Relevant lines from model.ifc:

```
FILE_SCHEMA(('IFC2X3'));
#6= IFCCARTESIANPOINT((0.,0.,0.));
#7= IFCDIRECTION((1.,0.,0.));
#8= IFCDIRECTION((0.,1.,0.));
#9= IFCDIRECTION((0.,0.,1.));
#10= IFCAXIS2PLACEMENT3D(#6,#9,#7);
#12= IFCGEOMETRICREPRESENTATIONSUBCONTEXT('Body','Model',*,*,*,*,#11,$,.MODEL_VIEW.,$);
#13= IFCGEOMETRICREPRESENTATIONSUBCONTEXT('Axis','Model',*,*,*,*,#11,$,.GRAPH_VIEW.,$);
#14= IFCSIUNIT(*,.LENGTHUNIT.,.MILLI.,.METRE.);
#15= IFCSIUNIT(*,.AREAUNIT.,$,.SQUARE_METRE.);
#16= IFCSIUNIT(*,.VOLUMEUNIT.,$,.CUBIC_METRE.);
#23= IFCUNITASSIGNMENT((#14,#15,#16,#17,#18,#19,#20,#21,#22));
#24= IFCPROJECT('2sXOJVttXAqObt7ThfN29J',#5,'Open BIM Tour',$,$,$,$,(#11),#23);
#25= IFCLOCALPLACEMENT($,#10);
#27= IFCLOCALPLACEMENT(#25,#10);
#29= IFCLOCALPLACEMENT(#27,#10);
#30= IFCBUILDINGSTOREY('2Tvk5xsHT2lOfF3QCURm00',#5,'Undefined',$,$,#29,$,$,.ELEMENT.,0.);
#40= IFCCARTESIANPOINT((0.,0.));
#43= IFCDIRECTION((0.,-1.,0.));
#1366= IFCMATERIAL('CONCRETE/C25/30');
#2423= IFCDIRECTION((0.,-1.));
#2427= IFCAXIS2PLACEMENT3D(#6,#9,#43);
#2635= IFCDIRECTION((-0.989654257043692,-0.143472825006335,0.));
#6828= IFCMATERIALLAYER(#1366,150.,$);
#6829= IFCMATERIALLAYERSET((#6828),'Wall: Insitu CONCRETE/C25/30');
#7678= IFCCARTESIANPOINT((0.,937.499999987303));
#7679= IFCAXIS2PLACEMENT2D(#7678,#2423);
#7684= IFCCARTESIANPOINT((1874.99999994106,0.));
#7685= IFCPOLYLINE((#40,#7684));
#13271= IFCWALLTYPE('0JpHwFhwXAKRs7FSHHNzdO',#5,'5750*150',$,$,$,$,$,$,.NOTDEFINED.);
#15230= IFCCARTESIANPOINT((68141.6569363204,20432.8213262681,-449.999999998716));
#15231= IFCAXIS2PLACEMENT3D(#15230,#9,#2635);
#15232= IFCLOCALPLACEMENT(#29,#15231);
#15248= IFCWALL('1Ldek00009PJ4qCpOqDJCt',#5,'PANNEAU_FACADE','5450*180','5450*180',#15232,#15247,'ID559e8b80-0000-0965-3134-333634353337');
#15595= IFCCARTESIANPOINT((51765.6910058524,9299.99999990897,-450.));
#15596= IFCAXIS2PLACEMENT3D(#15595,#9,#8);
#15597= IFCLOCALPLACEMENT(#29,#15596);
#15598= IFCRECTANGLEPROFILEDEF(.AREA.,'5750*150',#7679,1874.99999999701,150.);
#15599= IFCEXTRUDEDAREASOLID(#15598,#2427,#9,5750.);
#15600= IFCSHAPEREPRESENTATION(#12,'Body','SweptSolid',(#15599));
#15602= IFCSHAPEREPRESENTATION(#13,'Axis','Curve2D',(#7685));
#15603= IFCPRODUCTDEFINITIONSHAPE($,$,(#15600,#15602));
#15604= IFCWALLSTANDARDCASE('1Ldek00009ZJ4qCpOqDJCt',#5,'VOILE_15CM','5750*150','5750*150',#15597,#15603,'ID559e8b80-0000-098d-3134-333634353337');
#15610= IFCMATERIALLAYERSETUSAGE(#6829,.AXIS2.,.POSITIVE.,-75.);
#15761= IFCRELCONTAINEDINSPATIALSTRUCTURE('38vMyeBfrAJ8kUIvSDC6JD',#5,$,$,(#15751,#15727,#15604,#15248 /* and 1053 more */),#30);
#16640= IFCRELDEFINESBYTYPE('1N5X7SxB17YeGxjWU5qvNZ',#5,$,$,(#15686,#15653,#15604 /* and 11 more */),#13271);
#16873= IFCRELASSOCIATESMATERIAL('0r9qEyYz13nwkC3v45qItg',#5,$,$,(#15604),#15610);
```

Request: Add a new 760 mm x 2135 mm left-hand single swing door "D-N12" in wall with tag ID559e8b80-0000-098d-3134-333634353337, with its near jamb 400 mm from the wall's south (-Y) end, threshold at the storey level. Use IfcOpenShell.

```python
import numpy as np
import ifcopenshell
import ifcopenshell.api.feature
import ifcopenshell.api.geometry
import ifcopenshell.api.root
import ifcopenshell.api.spatial
import ifcopenshell.api.type
import ifcopenshell.geom
import ifcopenshell.util.element
import ifcopenshell.util.placement
import ifcopenshell.util.representation
import ifcopenshell.util.shape
import ifcopenshell.util.unit

model = ifcopenshell.open("model.ifc")
unit_scale = ifcopenshell.util.unit.calculate_unit_scale(model)
settings = ifcopenshell.geom.settings()


def volume(element):
    """Net volume in cubic metres, openings subtracted."""
    shape = ifcopenshell.geom.create_shape(settings, element)
    return ifcopenshell.util.shape.get_volume(shape.geometry)


wall = model.by_guid("1Ldek00009ZJ4qCpOqDJCt")
storey = ifcopenshell.util.element.get_container(wall, ifc_class="IfcBuildingStorey")
context = ifcopenshell.util.representation.get_context(model, "Model", "Body", "MODEL_VIEW")
before = volume(wall)

width, height, from_end, sill = 0.76, 2.135, 0.4, 0.0  # metres

# The wall runs along its own X axis, and the end named is its -X end.
wall_shape = ifcopenshell.geom.create_shape(settings, wall)
x, y, z = ifcopenshell.util.shape.get_vertices(wall_shape.geometry).T
start = x.min() + from_end
face, thickness = float(y.min()), float(y.max() - y.min())
wall_matrix = ifcopenshell.util.placement.get_local_placement(wall.ObjectPlacement)
level = ifcopenshell.util.placement.get_local_placement(storey.ObjectPlacement)[2, 3]


def in_wall(x, y):
    """Placement at x, y metres in the wall's axes, at sill height."""
    matrix = wall_matrix.copy()
    matrix[:, 3] = wall_matrix @ np.array([x / unit_scale, y / unit_scale, 0.0, 1.0])
    matrix[2, 3] = level + sill / unit_scale
    return matrix


# Opening: a box that overshoots both wall faces by 50 mm.
opening = ifcopenshell.api.root.create_entity(model, ifc_class="IfcOpeningElement")
box = ifcopenshell.api.geometry.add_wall_representation(
    model, context=context, length=width, height=height, thickness=thickness + 0.1
)
ifcopenshell.api.geometry.assign_representation(model, product=opening, representation=box)
ifcopenshell.api.geometry.edit_object_placement(model, product=opening, matrix=in_wall(start, face - 0.05), is_si=False)
ifcopenshell.api.feature.add_feature(model, feature=opening, element=wall)

door = ifcopenshell.api.root.create_entity(model, ifc_class="IfcDoor", name="D-N12")
door.OverallWidth, door.OverallHeight = width / unit_scale, height / unit_scale
body = ifcopenshell.api.geometry.add_door_representation(
    model,
    context=context,
    overall_width=door.OverallWidth,
    overall_height=door.OverallHeight,
    operation_type="SINGLE_SWING_LEFT",
    lining_properties={"LiningDepth": thickness / unit_scale, "ThresholdDepth": thickness / unit_scale},
)
ifcopenshell.api.geometry.assign_representation(model, product=door, representation=body)
ifcopenshell.api.spatial.assign_container(model, products=[door], relating_structure=storey)
fills = ifcopenshell.api.feature.add_filling(model, opening=opening, element=door)
fills.OwnerHistory = door.OwnerHistory  # required in IFC2X3

# IFC2X3 keeps the operation on the door style.
style = ifcopenshell.api.root.create_entity(model, ifc_class="IfcDoorStyle", name="D-N12")
style.OperationType, style.ConstructionType = "SINGLE_SWING_LEFT", "NOTDEFINED"
style.ParameterTakesPrecedence = style.Sizeable = False
ifcopenshell.api.type.assign_type(model, related_objects=[door], relating_type=style)

# The lining spans the wall, so the door starts at the wall face.
ifcopenshell.api.geometry.edit_object_placement(model, product=door, matrix=in_wall(start, face), is_si=False)

after = volume(wall)

print(f"wall volume {before:.3f} -> {after:.3f} m3")

model.write("model_updated.ifc")
```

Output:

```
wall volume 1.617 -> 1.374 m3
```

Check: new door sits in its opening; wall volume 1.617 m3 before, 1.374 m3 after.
